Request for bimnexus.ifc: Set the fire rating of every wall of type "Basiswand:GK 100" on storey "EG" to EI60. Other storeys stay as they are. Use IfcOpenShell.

First a look at what the model holds.

```python
import ifcopenshell
import ifcopenshell.util.element

model = ifcopenshell.open("bimnexus.ifc")
print(model.schema)
storey = next(s for s in model.by_type("IfcBuildingStorey") if s.Name == "EG")
walls = [e for e in ifcopenshell.util.element.get_decomposition(storey) if e.is_a("IfcWall")]
seen = {}
for e in walls:
    element_type = ifcopenshell.util.element.get_type(e)
    key = (element_type.Name if element_type != e and element_type else None, ifcopenshell.util.element.get_pset(e, "Pset_WallCommon", "FireRating"))
    seen[key] = seen.get(key, 0) + 1
for (name, value), count in sorted(seen.items(), key=str):
    print(count, "x", name, "|", value)
```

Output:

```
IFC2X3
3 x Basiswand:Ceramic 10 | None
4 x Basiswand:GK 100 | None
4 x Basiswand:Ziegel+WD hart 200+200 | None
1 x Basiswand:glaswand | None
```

```python
import ifcopenshell
import ifcopenshell.api.pset
import ifcopenshell.util.element

model = ifcopenshell.open("bimnexus.ifc")

storey = next(s for s in model.by_type("IfcBuildingStorey") if s.Name == "EG")
walls = [e for e in ifcopenshell.util.element.get_decomposition(storey) if e.is_a("IfcWall")]

count = 0
for e in walls:
    element_type = ifcopenshell.util.element.get_type(e)
    if element_type in (None, e) or element_type.Name != "Basiswand:GK 100":
        continue
    # add_pset returns the element's existing set when there is one.
    pset = ifcopenshell.api.pset.add_pset(model, product=e, name="Pset_WallCommon")
    ifcopenshell.api.pset.edit_pset(model, pset=pset, properties={"FireRating": "EI60"})
    count += 1

print(count, "walls updated")

model.write("bimnexus_edited.ifc")
```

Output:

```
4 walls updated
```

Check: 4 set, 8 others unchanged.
